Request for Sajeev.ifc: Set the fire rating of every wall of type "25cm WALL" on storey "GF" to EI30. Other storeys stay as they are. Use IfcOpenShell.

First a look at what the model holds.

```python
import ifcopenshell
import ifcopenshell.util.element

model = ifcopenshell.open("Sajeev.ifc")
print(model.schema)
storey = next(s for s in model.by_type("IfcBuildingStorey") if s.Name == "GF")
walls = [e for e in ifcopenshell.util.element.get_decomposition(storey) if e.is_a("IfcWall")]
seen = {}
for e in walls:
    element_type = ifcopenshell.util.element.get_type(e)
    key = (element_type.Name if element_type != e and element_type else None, ifcopenshell.util.element.get_pset(e, "Pset_WallCommon", "FireRating"))
    seen[key] = seen.get(key, 0) + 1
for (name, value), count in sorted(seen.items(), key=str):
    print(count, "x", name, "|", value)
```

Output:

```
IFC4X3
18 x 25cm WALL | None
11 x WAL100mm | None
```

```python
import ifcopenshell
import ifcopenshell.api.pset
import ifcopenshell.util.element

model = ifcopenshell.open("Sajeev.ifc")

storey = next(s for s in model.by_type("IfcBuildingStorey") if s.Name == "GF")
walls = [e for e in ifcopenshell.util.element.get_decomposition(storey) if e.is_a("IfcWall")]

count = 0
for e in walls:
    element_type = ifcopenshell.util.element.get_type(e)
    if element_type in (None, e) or element_type.Name != "25cm WALL":
        continue
    # add_pset returns the element's existing set when there is one.
    pset = ifcopenshell.api.pset.add_pset(model, product=e, name="Pset_WallCommon")
    ifcopenshell.api.pset.edit_pset(model, pset=pset, properties={"FireRating": "EI30"})
    count += 1

print(count, "walls updated")

model.write("Sajeev_v2.ifc")
```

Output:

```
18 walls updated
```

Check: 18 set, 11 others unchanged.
